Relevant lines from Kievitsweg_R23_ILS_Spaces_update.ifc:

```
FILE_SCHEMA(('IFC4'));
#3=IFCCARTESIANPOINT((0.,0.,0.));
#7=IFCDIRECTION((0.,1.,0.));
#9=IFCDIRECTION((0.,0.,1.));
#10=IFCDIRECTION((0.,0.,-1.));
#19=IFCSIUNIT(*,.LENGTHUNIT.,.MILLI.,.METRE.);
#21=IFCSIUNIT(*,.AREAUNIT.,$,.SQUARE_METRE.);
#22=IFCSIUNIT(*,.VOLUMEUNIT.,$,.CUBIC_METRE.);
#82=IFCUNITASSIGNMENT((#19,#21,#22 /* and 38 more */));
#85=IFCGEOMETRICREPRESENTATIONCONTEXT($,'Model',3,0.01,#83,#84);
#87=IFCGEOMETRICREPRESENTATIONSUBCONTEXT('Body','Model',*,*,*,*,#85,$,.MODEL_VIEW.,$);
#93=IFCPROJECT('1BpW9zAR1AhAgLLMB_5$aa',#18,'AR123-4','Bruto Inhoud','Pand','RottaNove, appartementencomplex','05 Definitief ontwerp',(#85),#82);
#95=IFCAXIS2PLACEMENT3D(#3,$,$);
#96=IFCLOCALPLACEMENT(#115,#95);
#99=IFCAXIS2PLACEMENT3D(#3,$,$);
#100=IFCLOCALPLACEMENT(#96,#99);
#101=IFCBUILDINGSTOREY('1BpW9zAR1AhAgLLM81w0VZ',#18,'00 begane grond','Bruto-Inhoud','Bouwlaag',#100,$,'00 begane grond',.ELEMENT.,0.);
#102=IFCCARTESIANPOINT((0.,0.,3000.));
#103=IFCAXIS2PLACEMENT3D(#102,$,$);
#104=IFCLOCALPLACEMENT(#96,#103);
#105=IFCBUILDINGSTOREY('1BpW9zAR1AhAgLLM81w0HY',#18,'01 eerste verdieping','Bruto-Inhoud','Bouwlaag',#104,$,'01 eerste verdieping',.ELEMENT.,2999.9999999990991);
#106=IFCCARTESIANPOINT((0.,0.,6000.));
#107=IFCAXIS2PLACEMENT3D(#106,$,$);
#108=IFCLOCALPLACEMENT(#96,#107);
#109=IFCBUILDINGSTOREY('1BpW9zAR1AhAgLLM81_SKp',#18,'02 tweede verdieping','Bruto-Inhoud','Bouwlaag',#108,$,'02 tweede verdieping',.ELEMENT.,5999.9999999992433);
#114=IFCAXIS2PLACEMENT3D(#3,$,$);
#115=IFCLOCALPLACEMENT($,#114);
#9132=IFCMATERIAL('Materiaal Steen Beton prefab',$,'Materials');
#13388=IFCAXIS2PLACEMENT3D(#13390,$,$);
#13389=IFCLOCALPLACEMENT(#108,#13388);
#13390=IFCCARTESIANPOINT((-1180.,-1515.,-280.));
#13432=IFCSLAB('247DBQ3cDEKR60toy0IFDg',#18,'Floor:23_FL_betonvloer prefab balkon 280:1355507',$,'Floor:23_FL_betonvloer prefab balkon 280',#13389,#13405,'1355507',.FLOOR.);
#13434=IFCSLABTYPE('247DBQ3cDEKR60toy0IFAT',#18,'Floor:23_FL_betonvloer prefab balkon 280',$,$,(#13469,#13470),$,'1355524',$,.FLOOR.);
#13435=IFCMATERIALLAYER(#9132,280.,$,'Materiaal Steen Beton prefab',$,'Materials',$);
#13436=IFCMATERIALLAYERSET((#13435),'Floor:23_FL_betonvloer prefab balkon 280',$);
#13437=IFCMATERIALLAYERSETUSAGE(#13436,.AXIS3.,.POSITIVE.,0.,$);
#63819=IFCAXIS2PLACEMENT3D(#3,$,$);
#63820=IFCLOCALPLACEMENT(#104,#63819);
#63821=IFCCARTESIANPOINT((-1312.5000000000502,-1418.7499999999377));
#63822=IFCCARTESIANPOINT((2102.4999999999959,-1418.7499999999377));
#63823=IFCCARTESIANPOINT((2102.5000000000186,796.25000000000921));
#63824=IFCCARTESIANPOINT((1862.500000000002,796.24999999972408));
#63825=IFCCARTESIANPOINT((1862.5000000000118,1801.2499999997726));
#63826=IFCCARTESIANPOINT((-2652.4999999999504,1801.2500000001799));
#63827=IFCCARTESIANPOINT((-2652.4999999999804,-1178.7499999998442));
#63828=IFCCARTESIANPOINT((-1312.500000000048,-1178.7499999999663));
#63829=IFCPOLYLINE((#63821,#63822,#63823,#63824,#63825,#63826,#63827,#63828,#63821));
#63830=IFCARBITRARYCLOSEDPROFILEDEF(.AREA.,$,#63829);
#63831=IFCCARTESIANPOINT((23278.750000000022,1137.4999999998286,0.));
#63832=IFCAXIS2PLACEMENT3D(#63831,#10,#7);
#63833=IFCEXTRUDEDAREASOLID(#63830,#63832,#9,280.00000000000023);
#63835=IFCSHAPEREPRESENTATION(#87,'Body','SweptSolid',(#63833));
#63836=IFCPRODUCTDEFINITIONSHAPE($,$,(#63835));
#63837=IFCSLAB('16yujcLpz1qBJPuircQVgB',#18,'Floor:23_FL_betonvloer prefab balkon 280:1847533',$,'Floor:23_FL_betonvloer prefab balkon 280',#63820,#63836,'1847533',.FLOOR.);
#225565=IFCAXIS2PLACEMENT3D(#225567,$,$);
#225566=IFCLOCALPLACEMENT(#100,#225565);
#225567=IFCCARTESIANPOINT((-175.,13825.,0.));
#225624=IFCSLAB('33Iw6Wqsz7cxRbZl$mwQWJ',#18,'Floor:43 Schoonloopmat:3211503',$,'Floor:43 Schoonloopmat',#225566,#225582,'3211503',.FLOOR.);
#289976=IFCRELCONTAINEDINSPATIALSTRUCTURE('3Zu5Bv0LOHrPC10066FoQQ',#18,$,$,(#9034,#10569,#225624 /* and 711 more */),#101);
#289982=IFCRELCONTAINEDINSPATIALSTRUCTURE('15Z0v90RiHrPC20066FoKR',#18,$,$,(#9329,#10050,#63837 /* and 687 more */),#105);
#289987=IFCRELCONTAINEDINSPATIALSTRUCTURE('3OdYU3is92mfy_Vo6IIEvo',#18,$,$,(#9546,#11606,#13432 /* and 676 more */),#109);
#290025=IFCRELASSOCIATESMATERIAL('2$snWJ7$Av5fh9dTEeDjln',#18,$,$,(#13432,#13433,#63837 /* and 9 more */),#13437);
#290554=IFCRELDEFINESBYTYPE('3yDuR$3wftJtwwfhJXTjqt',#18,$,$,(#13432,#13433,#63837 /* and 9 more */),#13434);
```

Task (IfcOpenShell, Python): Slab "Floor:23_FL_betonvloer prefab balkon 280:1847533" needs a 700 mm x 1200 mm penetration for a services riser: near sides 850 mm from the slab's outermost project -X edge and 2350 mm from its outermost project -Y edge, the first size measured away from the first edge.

```python
import numpy as np
import ifcopenshell
import ifcopenshell.api.feature
import ifcopenshell.api.geometry
import ifcopenshell.api.root
import ifcopenshell.geom
import ifcopenshell.util.placement
import ifcopenshell.util.representation
import ifcopenshell.util.shape
import ifcopenshell.util.unit

model = ifcopenshell.open("Kievitsweg_R23_ILS_Spaces_update.ifc")
unit_scale = ifcopenshell.util.unit.calculate_unit_scale(model)
settings = ifcopenshell.geom.settings()


def volume(element):
    """Net volume in cubic metres, openings subtracted."""
    shape = ifcopenshell.geom.create_shape(settings, element)
    return ifcopenshell.util.shape.get_volume(shape.geometry)


slab = model.by_guid("16yujcLpz1qBJPuircQVgB")
before = volume(slab)

# Extent in the slab's own axes, in metres. The edges named are its -X and -Y sides.
slab_shape = ifcopenshell.geom.create_shape(settings, slab)
vertices = ifcopenshell.util.shape.get_vertices(slab_shape.geometry)
x_min, y_min, bottom = vertices.min(axis=0)
top = vertices[:, 2].max()

opening = ifcopenshell.api.root.create_entity(model, ifc_class="IfcOpeningElement", name="Services riser opening", predefined_type="OPENING")
context = ifcopenshell.util.representation.get_context(model, "Model", "Body", "MODEL_VIEW")
width, depth = 0.7, 1.2
outline = [(0.0, 0.0), (width, 0.0), (width, depth), (0.0, depth), (0.0, 0.0)]
# Overshoot both faces by 50 mm so the cut is clean.
shape = ifcopenshell.api.geometry.add_slab_representation(
    model, context=context, depth=top - bottom + 0.1, polyline=outline
)
ifcopenshell.api.geometry.assign_representation(model, product=opening, representation=shape)

matrix = ifcopenshell.util.placement.get_local_placement(slab.ObjectPlacement)
matrix[:, 3] = matrix @ np.append(np.array([x_min + 0.85, y_min + 2.35, bottom - 0.05]) / unit_scale, 1.0)
ifcopenshell.api.geometry.edit_object_placement(model, product=opening, matrix=matrix, is_si=False)
ifcopenshell.api.feature.add_feature(model, feature=opening, element=slab)

after = volume(slab)

print(f"slab volume {before:.3f} -> {after:.3f} m3")

model.write("Kievitsweg_R23_ILS_Spaces_update-out.ifc")
```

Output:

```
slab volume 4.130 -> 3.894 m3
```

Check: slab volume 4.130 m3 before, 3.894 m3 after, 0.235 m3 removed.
